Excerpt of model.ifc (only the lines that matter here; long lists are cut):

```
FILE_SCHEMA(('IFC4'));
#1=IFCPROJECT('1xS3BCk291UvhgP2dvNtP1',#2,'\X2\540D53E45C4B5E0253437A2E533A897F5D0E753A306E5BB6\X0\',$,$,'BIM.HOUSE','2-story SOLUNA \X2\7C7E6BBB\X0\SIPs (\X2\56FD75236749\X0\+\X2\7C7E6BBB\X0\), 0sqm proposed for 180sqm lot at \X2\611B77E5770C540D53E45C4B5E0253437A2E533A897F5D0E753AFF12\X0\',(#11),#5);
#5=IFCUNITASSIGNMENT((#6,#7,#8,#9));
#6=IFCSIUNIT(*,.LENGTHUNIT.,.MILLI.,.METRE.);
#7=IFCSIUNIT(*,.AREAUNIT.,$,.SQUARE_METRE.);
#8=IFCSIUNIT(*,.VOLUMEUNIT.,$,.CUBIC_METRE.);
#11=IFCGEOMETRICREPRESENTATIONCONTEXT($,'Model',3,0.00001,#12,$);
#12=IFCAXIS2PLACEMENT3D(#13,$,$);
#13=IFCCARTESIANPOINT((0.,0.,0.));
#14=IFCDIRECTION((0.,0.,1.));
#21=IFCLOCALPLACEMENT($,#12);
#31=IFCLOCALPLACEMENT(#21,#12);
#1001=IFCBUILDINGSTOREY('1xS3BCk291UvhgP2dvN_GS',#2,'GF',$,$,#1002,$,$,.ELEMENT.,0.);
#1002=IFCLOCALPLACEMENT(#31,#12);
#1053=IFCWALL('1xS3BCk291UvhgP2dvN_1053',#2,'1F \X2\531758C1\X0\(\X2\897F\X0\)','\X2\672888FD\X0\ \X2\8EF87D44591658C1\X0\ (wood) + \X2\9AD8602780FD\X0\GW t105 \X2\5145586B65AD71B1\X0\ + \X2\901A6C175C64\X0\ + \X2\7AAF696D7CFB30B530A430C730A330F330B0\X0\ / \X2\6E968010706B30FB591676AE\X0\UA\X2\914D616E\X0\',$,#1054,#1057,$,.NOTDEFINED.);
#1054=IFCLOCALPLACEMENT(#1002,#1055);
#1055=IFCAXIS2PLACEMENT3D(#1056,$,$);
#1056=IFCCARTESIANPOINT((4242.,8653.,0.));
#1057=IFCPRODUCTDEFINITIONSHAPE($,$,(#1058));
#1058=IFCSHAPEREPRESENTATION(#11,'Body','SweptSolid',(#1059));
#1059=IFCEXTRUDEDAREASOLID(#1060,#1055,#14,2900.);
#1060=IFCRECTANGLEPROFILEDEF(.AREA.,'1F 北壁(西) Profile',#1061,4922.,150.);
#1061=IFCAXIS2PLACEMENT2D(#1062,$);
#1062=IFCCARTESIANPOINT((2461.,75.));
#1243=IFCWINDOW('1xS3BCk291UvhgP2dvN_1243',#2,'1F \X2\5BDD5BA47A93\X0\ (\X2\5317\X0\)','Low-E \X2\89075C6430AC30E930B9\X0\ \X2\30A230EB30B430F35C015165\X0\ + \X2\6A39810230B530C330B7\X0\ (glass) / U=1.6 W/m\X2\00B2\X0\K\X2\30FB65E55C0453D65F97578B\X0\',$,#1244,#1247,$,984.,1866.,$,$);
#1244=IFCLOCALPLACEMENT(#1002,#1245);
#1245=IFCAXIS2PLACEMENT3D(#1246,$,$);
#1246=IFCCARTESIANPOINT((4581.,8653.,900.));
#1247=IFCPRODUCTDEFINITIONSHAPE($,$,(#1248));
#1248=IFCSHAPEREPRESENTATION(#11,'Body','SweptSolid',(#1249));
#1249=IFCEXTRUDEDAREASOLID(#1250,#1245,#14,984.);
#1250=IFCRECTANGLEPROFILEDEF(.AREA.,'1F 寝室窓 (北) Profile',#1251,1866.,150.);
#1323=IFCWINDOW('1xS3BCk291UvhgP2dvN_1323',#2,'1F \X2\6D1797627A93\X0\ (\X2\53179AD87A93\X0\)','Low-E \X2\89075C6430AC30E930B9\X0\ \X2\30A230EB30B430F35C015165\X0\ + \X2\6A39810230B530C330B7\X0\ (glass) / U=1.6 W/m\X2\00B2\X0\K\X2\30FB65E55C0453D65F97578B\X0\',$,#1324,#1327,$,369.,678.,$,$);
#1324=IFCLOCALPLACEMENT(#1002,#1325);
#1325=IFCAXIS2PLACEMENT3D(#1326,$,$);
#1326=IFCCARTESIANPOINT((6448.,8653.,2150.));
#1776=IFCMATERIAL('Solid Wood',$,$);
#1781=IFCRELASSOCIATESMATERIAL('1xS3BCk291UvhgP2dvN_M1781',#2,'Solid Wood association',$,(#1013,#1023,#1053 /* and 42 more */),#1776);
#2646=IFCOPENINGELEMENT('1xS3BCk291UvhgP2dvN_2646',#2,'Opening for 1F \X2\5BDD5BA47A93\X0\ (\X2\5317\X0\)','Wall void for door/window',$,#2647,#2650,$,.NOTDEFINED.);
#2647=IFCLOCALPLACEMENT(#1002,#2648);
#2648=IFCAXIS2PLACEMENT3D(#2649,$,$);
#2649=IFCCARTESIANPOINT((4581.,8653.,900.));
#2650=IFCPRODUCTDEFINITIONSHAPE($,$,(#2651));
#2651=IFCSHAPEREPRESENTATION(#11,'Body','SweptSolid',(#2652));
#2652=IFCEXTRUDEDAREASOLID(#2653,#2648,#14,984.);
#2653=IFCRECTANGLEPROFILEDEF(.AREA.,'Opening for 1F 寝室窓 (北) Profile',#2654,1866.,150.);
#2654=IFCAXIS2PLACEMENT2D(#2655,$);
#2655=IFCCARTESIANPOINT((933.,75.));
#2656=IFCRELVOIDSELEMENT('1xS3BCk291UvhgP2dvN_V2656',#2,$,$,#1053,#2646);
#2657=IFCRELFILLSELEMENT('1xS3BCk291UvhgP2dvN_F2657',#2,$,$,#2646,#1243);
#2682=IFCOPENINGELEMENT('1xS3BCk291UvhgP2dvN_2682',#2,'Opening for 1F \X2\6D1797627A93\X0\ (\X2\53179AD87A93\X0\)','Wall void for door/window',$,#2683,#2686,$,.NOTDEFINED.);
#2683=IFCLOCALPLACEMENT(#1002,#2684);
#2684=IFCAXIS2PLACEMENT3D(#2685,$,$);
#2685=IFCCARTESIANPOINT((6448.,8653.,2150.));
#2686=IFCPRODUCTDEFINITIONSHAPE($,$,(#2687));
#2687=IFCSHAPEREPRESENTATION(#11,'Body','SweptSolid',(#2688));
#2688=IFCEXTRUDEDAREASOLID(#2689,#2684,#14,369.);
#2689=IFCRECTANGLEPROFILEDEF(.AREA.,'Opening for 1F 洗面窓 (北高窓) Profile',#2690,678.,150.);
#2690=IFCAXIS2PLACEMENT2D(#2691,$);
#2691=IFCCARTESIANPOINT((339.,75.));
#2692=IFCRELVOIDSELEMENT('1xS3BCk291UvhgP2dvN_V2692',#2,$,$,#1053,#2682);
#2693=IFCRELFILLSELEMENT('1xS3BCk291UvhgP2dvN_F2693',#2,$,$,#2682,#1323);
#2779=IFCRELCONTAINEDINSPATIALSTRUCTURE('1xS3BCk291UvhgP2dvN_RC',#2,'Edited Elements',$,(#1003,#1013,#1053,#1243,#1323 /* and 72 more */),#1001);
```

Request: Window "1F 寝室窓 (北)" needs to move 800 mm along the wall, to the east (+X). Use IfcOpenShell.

```python
import ifcopenshell
import ifcopenshell.api.geometry
import ifcopenshell.util.placement

model = ifcopenshell.open("model.ifc")

window = model.by_guid("1xS3BCk291UvhgP2dvN_1243")
opening = window.FillsVoids[0].RelatingOpeningElement
wall = opening.VoidsElements[0].RelatingBuildingElement

wall_matrix = ifcopenshell.util.placement.get_local_placement(wall.ObjectPlacement)
shift = wall_matrix[:3, 0] * 800.0
before = ifcopenshell.util.placement.get_local_placement(window.ObjectPlacement)[:3, 3].copy()

# The window is not placed relative to its opening, so move both.
for product in (opening, window):
    matrix = ifcopenshell.util.placement.get_local_placement(product.ObjectPlacement)
    matrix[:3, 3] += shift
    ifcopenshell.api.geometry.edit_object_placement(model, product=product, matrix=matrix, is_si=False)

after = ifcopenshell.util.placement.get_local_placement(window.ObjectPlacement)[:3, 3]
print("window moved by", (after - before).round(3) + 0.0)

model.write("model_edited.ifc")
```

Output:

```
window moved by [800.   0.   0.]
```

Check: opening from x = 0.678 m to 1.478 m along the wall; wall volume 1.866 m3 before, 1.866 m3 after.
